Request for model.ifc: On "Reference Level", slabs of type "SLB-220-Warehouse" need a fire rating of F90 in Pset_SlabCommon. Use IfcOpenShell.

First a look at what the model holds.

```python
import ifcopenshell
import ifcopenshell.util.element

model = ifcopenshell.open("model.ifc")
print(model.schema)
storey = next(s for s in model.by_type("IfcBuildingStorey") if s.Name == "Reference Level")
slabs = [e for e in ifcopenshell.util.element.get_decomposition(storey) if e.is_a("IfcSlab")]
seen = {}
for e in slabs:
    element_type = ifcopenshell.util.element.get_type(e)
    key = (element_type.Name if element_type != e and element_type else None, ifcopenshell.util.element.get_pset(e, "Pset_SlabCommon", "FireRating"))
    seen[key] = seen.get(key, 0) + 1
for (name, value), count in sorted(seen.items(), key=str):
    print(count, "x", name, "|", value)
```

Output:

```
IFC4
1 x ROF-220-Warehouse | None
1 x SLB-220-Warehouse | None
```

```python
import ifcopenshell
import ifcopenshell.api.pset
import ifcopenshell.util.element

model = ifcopenshell.open("model.ifc")

storey = next(s for s in model.by_type("IfcBuildingStorey") if s.Name == "Reference Level")
slabs = [e for e in ifcopenshell.util.element.get_decomposition(storey) if e.is_a("IfcSlab")]

count = 0
for e in slabs:
    element_type = ifcopenshell.util.element.get_type(e)
    if element_type in (None, e) or element_type.Name != "SLB-220-Warehouse":
        continue
    # add_pset returns the element's existing set when there is one.
    pset = ifcopenshell.api.pset.add_pset(model, product=e, name="Pset_SlabCommon")
    ifcopenshell.api.pset.edit_pset(model, pset=pset, properties={"FireRating": "F90"})
    count += 1

print(count, "slabs updated")

model.write("model_edited.ifc")
```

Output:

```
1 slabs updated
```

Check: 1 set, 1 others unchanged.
